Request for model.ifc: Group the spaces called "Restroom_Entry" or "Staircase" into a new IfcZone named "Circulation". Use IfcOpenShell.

First a look at what the model holds.

```python
import ifcopenshell

model = ifcopenshell.open("model.ifc")
print(model.schema)
seen = {}
for space in model.by_type("IfcSpace"):
    seen[space.LongName] = seen.get(space.LongName, 0) + 1
for name, count in sorted(seen.items(), key=str):
    print(count, "x", name)
print("zones:", [z.Name for z in model.by_type("IfcZone")][:20])
```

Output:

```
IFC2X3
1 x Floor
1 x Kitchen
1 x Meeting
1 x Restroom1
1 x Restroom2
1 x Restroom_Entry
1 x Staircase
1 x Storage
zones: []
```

```python
import ifcopenshell
import ifcopenshell.api.group
import ifcopenshell.api.root

model = ifcopenshell.open("model.ifc")

names = {"Restroom_Entry", "Staircase"}
spaces = [s for s in model.by_type("IfcSpace") if s.LongName in names]

zone = ifcopenshell.api.root.create_entity(model, ifc_class="IfcZone", name="Circulation")
ifcopenshell.api.group.assign_group(model, products=spaces, group=zone)
print(len(spaces), "spaces in", zone.Name)

model.write("model_edited.ifc")
```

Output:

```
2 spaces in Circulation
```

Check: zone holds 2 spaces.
